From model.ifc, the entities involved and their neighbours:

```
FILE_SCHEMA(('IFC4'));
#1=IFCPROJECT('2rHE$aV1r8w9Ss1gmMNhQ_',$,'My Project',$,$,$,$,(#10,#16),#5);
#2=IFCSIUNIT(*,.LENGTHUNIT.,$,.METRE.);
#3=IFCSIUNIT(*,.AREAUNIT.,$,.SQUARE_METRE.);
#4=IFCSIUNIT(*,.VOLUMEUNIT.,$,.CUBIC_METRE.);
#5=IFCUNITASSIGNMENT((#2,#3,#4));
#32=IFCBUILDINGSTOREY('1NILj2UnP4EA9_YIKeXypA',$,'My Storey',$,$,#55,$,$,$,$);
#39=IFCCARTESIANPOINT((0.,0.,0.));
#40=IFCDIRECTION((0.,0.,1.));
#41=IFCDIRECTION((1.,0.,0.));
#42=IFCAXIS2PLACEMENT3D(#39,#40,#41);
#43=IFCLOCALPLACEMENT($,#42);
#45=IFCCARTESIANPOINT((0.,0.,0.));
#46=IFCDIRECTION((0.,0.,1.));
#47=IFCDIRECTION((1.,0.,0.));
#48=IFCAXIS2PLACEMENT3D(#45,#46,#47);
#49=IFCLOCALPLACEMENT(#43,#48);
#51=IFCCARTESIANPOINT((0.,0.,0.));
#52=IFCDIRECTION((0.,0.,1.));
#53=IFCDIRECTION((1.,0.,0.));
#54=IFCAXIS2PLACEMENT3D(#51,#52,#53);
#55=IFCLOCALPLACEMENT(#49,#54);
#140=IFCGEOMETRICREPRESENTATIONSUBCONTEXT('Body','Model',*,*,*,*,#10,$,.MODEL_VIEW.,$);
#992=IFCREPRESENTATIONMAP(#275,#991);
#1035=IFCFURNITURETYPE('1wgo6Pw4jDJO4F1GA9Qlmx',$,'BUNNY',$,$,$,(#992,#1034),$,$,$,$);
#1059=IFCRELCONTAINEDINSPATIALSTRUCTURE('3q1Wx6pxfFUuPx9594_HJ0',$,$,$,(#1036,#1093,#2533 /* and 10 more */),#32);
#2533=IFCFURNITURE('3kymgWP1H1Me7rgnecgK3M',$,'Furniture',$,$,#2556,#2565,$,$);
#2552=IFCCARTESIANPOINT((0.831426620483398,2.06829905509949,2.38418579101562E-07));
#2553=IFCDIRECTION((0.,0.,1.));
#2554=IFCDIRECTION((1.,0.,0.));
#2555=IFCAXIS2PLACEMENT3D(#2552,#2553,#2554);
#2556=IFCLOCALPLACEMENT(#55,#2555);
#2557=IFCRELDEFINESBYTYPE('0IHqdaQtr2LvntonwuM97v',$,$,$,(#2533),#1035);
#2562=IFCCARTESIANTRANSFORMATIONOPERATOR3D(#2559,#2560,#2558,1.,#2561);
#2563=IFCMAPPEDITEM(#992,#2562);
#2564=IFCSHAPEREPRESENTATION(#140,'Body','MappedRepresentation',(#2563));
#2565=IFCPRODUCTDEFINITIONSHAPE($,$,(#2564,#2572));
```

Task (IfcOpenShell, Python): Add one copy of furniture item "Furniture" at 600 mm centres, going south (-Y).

```python
import numpy as np
import ifcopenshell
import ifcopenshell.api.geometry
import ifcopenshell.api.root
import ifcopenshell.util.element
import ifcopenshell.util.placement

model = ifcopenshell.open("model.ifc")

source = model.by_id(2533)
base = ifcopenshell.util.placement.get_local_placement(source.ObjectPlacement)
step = np.array([0.0, -1.0, 0.0]) * 0.6

for i in range(1, 2):
    copy = ifcopenshell.api.root.copy_class(model, product=source)
    copy.Representation = ifcopenshell.util.element.copy_deep(
        model, source.Representation, exclude=["IfcGeometricRepresentationContext", "IfcRepresentationMap"]
    )
    matrix = base.copy()
    matrix[:3, 3] += i * step
    print("added at", matrix[:3, 3].round(3) + 0.0)
    ifcopenshell.api.geometry.edit_object_placement(model, product=copy, matrix=matrix, is_si=False)

model.write("model_v2.ifc")
```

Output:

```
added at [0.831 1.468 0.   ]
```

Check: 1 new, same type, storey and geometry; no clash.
